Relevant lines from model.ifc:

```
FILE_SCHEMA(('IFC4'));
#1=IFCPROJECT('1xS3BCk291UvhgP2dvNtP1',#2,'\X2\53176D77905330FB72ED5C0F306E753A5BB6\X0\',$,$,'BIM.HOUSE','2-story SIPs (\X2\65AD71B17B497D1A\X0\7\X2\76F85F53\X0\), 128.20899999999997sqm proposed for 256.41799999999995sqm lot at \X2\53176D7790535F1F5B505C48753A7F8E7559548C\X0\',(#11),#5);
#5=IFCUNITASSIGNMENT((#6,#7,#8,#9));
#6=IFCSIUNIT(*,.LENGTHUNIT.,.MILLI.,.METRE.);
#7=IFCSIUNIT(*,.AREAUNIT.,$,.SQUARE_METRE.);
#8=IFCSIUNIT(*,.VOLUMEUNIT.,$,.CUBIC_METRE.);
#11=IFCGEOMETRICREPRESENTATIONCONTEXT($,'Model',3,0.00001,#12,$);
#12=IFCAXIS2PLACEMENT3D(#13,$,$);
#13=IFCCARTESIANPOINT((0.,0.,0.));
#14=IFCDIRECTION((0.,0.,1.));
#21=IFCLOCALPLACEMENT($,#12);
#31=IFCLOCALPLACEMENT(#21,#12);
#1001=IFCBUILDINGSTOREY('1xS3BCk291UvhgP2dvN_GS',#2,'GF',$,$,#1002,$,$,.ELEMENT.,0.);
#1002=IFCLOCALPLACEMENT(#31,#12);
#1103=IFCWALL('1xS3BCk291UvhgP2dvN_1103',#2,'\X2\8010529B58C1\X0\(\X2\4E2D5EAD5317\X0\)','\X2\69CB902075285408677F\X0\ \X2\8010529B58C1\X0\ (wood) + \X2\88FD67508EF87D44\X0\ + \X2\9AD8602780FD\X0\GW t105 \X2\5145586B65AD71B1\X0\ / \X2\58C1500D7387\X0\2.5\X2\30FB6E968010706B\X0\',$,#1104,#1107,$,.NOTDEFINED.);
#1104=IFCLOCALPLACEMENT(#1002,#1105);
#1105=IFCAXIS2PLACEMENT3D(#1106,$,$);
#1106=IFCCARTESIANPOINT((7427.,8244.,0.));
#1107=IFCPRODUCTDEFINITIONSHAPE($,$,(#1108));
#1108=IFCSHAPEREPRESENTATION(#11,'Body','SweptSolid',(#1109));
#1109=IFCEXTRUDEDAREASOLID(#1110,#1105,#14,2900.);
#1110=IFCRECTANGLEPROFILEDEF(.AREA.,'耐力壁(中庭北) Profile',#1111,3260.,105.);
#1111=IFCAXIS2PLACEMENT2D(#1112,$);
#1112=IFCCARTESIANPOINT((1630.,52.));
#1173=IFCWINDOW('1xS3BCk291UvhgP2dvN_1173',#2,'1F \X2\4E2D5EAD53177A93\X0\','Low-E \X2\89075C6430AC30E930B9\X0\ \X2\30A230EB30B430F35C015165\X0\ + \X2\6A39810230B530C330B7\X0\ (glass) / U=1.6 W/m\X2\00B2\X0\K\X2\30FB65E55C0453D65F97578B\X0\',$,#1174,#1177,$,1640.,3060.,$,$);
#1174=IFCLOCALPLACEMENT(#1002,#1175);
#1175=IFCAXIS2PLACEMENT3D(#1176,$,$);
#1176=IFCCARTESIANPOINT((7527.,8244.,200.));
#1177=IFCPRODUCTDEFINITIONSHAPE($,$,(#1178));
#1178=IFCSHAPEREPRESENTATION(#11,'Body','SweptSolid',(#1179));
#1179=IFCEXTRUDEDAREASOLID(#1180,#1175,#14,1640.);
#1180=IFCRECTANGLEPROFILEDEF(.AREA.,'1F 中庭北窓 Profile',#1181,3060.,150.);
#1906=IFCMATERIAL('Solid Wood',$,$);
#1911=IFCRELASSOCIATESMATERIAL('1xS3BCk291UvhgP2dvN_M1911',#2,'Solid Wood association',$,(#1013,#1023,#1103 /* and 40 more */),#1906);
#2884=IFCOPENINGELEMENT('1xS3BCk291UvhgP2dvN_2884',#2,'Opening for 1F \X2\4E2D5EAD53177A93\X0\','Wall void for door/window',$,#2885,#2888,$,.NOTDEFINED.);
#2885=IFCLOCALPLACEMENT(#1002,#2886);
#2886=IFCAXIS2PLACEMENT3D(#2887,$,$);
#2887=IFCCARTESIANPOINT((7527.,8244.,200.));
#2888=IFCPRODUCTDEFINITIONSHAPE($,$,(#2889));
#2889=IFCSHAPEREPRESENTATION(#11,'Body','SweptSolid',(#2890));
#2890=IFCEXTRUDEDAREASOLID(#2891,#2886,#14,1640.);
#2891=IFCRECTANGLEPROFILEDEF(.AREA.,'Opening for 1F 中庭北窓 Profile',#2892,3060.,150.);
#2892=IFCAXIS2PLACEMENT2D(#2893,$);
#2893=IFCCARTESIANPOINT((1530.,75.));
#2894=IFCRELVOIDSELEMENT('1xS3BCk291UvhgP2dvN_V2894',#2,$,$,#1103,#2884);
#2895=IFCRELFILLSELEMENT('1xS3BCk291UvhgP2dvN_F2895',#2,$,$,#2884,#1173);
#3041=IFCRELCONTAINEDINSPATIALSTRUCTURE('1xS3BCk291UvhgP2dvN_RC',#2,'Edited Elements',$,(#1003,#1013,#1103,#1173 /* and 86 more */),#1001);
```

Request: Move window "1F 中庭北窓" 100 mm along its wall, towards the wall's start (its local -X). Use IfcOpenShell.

```python
import ifcopenshell
import ifcopenshell.api.geometry
import ifcopenshell.util.placement
import ifcopenshell.util.unit

model = ifcopenshell.open("model.ifc")
unit_scale = ifcopenshell.util.unit.calculate_unit_scale(model)

window = model.by_guid("1xS3BCk291UvhgP2dvN_1173")
opening = window.FillsVoids[0].RelatingOpeningElement
wall = opening.VoidsElements[0].RelatingBuildingElement

wall_matrix = ifcopenshell.util.placement.get_local_placement(wall.ObjectPlacement)
shift = wall_matrix[:3, 0] * -0.1 / unit_scale
before = ifcopenshell.util.placement.get_local_placement(window.ObjectPlacement)[:3, 3].copy()

# The window is not placed relative to its opening, so move both.
for product in (opening, window):
    matrix = ifcopenshell.util.placement.get_local_placement(product.ObjectPlacement)
    matrix[:3, 3] += shift
    ifcopenshell.api.geometry.edit_object_placement(model, product=product, matrix=matrix, is_si=False)

after = ifcopenshell.util.placement.get_local_placement(window.ObjectPlacement)[:3, 3]
print("window moved by", (after - before).round(3) + 0.0)

model.write("model_updated.ifc")
```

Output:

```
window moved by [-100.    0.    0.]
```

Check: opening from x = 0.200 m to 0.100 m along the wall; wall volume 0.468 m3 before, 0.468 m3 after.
